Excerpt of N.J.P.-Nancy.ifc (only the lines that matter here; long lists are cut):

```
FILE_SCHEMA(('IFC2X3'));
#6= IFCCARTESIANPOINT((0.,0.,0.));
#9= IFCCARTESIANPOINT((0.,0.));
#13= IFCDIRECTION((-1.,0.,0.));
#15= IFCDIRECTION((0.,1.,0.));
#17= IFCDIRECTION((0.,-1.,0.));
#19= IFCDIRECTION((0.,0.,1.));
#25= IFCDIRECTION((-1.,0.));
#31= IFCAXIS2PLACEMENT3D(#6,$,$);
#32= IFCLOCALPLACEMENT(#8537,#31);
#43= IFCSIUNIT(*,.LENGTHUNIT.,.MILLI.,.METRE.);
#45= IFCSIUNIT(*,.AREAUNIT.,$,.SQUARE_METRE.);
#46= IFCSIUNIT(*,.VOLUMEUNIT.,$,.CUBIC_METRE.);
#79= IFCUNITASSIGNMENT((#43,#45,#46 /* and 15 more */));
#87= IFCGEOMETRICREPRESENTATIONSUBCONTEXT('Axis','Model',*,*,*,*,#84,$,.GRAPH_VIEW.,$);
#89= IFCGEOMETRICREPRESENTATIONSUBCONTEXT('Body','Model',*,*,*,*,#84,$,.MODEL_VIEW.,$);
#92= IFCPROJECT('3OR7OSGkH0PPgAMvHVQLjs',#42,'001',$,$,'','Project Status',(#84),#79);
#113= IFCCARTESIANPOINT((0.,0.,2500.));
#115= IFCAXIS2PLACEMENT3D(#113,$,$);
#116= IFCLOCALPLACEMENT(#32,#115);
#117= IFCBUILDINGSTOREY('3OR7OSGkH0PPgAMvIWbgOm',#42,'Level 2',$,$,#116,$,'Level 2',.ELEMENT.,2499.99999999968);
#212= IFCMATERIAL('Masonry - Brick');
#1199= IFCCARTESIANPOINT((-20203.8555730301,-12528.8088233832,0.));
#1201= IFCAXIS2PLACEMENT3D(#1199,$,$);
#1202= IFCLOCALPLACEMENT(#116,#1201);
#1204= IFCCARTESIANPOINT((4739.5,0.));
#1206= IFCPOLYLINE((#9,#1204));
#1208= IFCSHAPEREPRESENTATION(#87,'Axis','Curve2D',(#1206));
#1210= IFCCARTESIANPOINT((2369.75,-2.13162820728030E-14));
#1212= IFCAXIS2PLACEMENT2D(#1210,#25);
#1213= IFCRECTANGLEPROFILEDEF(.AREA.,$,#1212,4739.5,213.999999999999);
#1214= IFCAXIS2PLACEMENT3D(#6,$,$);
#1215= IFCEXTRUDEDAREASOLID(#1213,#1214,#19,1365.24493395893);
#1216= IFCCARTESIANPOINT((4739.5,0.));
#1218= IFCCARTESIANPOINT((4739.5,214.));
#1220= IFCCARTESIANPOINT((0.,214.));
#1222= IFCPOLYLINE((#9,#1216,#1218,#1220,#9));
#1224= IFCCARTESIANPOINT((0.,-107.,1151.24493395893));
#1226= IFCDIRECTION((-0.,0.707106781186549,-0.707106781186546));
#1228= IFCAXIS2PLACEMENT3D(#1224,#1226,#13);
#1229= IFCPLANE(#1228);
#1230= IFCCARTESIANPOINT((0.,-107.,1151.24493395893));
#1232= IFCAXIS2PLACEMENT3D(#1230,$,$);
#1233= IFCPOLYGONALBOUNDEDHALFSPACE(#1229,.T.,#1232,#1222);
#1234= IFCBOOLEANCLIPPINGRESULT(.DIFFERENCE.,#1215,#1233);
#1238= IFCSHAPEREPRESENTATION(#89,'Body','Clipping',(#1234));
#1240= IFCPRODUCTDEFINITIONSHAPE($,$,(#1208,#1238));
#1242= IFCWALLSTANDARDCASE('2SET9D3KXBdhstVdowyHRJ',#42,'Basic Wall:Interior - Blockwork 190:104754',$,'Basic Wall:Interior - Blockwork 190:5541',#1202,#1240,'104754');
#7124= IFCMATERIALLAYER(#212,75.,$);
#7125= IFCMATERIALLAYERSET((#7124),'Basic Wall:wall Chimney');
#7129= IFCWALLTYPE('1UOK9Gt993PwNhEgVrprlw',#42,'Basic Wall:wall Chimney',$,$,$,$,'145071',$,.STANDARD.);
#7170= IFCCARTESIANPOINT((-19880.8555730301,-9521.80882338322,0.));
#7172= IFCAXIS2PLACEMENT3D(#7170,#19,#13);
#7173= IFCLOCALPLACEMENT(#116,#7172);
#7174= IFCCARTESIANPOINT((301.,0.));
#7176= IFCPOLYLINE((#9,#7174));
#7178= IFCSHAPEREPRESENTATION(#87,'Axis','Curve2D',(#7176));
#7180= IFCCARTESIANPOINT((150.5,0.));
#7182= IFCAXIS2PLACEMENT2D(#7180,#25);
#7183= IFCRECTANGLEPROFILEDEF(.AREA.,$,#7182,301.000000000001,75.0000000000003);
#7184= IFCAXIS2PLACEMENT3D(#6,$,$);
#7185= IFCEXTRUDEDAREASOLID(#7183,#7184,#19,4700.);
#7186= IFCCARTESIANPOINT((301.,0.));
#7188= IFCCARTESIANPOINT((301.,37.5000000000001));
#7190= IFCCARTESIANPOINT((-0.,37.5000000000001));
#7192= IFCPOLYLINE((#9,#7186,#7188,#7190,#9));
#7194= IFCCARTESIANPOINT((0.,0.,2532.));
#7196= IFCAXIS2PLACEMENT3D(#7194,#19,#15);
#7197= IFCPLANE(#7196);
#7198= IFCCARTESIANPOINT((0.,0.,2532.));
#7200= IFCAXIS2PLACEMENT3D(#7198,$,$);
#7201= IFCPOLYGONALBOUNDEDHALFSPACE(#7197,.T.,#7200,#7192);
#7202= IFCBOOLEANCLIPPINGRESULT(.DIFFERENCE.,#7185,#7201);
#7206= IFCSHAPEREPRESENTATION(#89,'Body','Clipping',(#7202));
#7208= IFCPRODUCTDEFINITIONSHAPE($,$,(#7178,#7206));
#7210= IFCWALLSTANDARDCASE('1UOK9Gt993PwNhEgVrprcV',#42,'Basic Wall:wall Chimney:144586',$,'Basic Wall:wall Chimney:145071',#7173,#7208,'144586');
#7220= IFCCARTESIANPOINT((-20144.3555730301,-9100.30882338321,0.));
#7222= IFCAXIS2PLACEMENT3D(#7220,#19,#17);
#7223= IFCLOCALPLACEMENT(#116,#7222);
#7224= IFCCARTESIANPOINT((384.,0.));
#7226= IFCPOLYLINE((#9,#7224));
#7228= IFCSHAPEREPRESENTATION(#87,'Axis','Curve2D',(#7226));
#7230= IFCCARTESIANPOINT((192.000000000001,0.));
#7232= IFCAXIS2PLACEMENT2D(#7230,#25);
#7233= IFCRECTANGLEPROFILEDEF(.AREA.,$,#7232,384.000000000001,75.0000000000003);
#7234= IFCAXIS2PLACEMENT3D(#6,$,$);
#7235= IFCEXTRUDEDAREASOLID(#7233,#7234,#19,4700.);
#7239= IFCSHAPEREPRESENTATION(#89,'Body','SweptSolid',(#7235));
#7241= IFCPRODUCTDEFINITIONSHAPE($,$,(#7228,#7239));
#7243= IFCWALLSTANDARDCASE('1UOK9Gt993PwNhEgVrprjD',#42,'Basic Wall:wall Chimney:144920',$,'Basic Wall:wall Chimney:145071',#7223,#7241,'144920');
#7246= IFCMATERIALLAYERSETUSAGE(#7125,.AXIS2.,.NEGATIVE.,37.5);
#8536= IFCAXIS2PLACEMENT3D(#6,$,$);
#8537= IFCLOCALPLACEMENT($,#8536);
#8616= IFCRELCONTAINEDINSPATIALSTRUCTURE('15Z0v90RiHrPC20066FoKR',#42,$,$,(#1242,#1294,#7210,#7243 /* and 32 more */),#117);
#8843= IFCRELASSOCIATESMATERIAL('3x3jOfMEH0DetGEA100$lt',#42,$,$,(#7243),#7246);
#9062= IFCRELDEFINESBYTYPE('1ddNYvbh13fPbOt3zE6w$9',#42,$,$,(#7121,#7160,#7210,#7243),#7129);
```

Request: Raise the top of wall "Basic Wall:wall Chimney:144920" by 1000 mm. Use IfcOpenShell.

```python
import ifcopenshell
import ifcopenshell.geom
import ifcopenshell.util.representation
import ifcopenshell.util.shape

model = ifcopenshell.open("N.J.P.-Nancy.ifc")
settings = ifcopenshell.geom.settings()


def volume(element):
    """Net volume in cubic metres, openings subtracted."""
    shape = ifcopenshell.geom.create_shape(settings, element)
    return ifcopenshell.util.shape.get_volume(shape.geometry)


wall = model.by_guid("1UOK9Gt993PwNhEgVrprjD")
before = volume(wall)

body = ifcopenshell.util.representation.get_representation(wall, "Model", "Body")
solid = body.Items[0]
old_height = solid.Depth
solid.Depth += 1000.0
after = volume(wall)

print(f"height {old_height:g} -> {solid.Depth:g}, volume {before:.3f} -> {after:.3f} m3")

model.write("N.J.P.-Nancy_updated.ifc")
```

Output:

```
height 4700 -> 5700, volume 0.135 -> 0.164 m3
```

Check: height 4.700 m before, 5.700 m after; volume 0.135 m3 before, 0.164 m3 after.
